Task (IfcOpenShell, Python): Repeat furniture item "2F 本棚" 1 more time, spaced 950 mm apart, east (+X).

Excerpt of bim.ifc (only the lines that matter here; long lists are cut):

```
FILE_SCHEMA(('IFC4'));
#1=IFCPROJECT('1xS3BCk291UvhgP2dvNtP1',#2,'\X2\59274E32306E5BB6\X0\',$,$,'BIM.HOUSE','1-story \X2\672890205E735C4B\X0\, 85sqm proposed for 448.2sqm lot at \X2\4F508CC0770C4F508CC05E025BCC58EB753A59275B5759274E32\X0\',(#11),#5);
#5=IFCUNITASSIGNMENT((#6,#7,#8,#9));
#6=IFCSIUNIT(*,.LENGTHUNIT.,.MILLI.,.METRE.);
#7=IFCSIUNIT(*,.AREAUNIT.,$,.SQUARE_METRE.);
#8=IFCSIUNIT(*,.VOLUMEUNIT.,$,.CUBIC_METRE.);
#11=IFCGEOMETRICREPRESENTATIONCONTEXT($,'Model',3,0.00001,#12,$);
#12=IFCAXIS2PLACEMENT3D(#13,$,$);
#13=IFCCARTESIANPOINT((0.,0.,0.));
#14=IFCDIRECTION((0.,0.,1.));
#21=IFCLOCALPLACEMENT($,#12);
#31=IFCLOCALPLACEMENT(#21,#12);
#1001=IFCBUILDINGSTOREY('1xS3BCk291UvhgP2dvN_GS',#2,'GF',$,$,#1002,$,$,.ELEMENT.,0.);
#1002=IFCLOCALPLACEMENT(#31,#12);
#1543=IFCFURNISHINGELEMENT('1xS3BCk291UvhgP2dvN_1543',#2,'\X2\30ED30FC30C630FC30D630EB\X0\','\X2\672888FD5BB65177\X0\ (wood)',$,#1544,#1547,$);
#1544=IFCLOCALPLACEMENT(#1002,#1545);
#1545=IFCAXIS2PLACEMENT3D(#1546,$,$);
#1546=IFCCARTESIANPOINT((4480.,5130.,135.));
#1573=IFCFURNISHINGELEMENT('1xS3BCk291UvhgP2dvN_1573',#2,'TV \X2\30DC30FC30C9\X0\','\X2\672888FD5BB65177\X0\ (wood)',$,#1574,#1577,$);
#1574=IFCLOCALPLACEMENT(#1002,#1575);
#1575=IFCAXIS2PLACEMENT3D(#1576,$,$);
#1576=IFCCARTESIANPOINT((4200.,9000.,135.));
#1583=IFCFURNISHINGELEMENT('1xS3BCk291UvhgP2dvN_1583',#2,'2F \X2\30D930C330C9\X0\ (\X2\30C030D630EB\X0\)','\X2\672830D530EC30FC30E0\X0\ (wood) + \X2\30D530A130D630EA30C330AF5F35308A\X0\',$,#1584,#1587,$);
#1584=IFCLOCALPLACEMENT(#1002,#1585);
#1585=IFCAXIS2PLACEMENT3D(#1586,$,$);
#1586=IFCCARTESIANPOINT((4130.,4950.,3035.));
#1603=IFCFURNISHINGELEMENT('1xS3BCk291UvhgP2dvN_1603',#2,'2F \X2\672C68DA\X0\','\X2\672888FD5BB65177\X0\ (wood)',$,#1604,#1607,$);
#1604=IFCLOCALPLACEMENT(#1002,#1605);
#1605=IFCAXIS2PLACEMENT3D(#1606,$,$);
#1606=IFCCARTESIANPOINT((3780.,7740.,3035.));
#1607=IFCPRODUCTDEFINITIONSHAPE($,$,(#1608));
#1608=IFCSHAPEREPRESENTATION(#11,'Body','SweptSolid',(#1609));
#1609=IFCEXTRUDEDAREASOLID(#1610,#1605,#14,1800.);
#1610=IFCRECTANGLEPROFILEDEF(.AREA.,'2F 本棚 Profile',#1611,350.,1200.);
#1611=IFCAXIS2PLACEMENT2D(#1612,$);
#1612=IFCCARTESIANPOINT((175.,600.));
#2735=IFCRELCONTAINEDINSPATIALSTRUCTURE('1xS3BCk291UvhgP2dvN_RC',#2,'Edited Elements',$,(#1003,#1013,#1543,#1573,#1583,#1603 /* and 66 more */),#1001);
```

```python
import numpy as np
import ifcopenshell
import ifcopenshell.api.geometry
import ifcopenshell.api.root
import ifcopenshell.util.element
import ifcopenshell.util.placement
import ifcopenshell.util.unit

model = ifcopenshell.open("bim.ifc")
unit_scale = ifcopenshell.util.unit.calculate_unit_scale(model)


def reuse_history(source, copy):
    """copy_class also copies each property set's owner history, people and application; keep the originals."""
    for rel in copy.IsDefinedBy:
        if rel.is_a("IfcRelDefinesByProperties") and (history := rel.RelatingPropertyDefinition.OwnerHistory):
            rel.RelatingPropertyDefinition.OwnerHistory = source.OwnerHistory
            ifcopenshell.util.element.remove_deep2(model, history)


source = model.by_guid("1xS3BCk291UvhgP2dvN_1603")
base = ifcopenshell.util.placement.get_local_placement(source.ObjectPlacement)
step = np.array([1.0, 0.0, 0.0]) * 0.95 / unit_scale

for i in range(1, 2):
    copy = ifcopenshell.api.root.copy_class(model, product=source)
    copy.Representation = ifcopenshell.util.element.copy_deep(
        model, source.Representation, exclude=["IfcGeometricRepresentationContext", "IfcRepresentationMap"]
    )
    reuse_history(source, copy)
    matrix = base.copy()
    matrix[:3, 3] += i * step
    print("added at", matrix[:3, 3].round(3) + 0.0)
    ifcopenshell.api.geometry.edit_object_placement(model, product=copy, matrix=matrix, is_si=False)

model.write("bim_v2.ifc")
```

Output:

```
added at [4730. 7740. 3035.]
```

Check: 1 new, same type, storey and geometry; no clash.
